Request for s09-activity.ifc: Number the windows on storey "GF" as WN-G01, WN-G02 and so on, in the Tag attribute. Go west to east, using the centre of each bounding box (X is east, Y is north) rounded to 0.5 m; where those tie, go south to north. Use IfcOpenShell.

First a look at what the model holds.

```python
import ifcopenshell
import ifcopenshell.util.element
import ifcopenshell.util.placement

model = ifcopenshell.open("s09-activity.ifc")
print(model.schema)
storey = next(s for s in model.by_type("IfcBuildingStorey") if s.Name == "GF")
windows = [e for e in ifcopenshell.util.element.get_decomposition(storey) if e.is_a("IfcWindow")]
for e in sorted(windows, key=lambda e: e.id()):
    origin = ifcopenshell.util.placement.get_local_placement(e.ObjectPlacement)[:3, 3]
    print(e.id(), e.Tag, e.Name, origin.round(2) + 0.0, sep=" | ")
```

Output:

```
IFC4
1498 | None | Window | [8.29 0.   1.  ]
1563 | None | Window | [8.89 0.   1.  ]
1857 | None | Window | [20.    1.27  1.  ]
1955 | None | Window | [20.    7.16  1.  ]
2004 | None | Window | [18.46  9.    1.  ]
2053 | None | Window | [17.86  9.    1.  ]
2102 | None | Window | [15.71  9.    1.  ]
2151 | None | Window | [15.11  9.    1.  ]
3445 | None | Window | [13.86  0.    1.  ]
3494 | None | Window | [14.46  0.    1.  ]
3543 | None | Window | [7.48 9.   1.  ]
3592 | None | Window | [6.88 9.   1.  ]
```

```python
import ifcopenshell
import ifcopenshell.geom
import ifcopenshell.util.element
import ifcopenshell.util.shape

model = ifcopenshell.open("s09-activity.ifc")
settings = ifcopenshell.geom.settings()
settings.set("use-world-coords", True)


def centre(element):
    shape = ifcopenshell.geom.create_shape(settings, element)
    return ifcopenshell.util.shape.get_bbox_centroid(shape.geometry)


storey = next(s for s in model.by_type("IfcBuildingStorey") if s.Name == "GF")
windows = [e for e in ifcopenshell.util.element.get_decomposition(storey) if e.is_a("IfcWindow")]

# Insertion points can sit at a corner or the storey origin, so sort by the geometry (in metres).
centres = {e: centre(e) for e in windows}
windows.sort(key=lambda e: (round(centres[e][0] / 0.5), centres[e][1]))

for i, e in enumerate(windows, start=1):
    number = f"WN-G{i:02d}"
    e.Tag = number
    print(e.id(), number)

model.write("s09-activity_edited.ifc")
```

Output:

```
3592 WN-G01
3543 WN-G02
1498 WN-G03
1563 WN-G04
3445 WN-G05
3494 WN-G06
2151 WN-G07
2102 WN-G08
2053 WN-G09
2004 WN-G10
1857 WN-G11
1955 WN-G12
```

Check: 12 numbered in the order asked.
